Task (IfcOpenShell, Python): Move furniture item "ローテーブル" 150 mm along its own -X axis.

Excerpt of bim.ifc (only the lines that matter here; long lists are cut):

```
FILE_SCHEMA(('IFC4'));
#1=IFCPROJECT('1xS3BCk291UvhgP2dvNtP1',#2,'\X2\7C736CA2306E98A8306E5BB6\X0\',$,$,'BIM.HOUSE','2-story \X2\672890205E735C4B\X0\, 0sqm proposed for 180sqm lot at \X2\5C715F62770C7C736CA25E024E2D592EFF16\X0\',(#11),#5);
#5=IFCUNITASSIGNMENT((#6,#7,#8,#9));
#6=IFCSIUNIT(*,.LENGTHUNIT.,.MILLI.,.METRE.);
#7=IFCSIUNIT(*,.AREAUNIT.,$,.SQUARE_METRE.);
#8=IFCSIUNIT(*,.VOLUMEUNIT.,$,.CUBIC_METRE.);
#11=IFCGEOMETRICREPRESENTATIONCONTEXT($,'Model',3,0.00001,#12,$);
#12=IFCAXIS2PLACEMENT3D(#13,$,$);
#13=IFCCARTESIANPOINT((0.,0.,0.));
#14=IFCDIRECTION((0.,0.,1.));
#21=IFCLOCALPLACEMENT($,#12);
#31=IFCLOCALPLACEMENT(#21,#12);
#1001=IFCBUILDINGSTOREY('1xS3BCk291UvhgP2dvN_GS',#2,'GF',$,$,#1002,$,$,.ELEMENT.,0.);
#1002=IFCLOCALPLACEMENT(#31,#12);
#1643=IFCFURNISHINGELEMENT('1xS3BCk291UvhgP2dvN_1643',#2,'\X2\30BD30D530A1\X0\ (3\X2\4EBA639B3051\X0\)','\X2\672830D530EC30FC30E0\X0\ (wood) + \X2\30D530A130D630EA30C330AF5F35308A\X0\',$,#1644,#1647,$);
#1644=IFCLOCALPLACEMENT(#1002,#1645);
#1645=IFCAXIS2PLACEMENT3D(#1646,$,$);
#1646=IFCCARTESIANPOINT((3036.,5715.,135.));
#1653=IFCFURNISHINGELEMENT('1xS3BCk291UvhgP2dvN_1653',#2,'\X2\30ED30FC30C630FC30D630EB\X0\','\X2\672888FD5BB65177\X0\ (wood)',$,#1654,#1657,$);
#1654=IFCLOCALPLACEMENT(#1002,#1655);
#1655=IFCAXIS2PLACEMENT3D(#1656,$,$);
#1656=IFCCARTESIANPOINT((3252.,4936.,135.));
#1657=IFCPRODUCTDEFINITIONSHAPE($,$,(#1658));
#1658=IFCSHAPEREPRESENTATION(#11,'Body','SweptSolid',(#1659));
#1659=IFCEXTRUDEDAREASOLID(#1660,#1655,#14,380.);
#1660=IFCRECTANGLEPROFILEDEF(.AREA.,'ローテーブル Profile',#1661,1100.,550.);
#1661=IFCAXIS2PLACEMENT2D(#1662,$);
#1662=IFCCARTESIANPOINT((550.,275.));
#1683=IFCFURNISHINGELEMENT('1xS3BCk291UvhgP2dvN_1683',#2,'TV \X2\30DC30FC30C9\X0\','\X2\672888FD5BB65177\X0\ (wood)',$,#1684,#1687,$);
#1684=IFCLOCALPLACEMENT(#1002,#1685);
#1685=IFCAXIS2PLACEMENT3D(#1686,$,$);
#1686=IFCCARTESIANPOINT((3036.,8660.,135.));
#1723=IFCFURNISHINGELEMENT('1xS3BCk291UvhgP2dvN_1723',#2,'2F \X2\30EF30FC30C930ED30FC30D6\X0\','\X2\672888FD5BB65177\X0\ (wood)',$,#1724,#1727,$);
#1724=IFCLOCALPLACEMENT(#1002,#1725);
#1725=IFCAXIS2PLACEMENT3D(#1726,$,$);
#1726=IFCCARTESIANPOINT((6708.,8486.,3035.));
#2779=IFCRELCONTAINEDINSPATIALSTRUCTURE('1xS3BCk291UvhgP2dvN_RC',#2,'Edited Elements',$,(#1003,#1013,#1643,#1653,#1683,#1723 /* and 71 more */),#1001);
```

```python
import ifcopenshell
import ifcopenshell.api.geometry
import ifcopenshell.util.placement

model = ifcopenshell.open("bim.ifc")

item = model.by_guid("1xS3BCk291UvhgP2dvN_1653")
matrix = ifcopenshell.util.placement.get_local_placement(item.ObjectPlacement)
matrix[:3, 3] -= matrix[:3, 0] * 150.0
ifcopenshell.api.geometry.edit_object_placement(model, product=item, matrix=matrix, is_si=False)

print(ifcopenshell.util.placement.get_local_placement(item.ObjectPlacement).round(3) + 0.0)

model.write("bim-out.ifc")
```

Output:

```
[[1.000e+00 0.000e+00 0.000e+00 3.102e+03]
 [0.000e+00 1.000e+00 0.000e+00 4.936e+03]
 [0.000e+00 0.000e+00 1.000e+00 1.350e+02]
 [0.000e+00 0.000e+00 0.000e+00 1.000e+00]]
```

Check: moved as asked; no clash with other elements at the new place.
